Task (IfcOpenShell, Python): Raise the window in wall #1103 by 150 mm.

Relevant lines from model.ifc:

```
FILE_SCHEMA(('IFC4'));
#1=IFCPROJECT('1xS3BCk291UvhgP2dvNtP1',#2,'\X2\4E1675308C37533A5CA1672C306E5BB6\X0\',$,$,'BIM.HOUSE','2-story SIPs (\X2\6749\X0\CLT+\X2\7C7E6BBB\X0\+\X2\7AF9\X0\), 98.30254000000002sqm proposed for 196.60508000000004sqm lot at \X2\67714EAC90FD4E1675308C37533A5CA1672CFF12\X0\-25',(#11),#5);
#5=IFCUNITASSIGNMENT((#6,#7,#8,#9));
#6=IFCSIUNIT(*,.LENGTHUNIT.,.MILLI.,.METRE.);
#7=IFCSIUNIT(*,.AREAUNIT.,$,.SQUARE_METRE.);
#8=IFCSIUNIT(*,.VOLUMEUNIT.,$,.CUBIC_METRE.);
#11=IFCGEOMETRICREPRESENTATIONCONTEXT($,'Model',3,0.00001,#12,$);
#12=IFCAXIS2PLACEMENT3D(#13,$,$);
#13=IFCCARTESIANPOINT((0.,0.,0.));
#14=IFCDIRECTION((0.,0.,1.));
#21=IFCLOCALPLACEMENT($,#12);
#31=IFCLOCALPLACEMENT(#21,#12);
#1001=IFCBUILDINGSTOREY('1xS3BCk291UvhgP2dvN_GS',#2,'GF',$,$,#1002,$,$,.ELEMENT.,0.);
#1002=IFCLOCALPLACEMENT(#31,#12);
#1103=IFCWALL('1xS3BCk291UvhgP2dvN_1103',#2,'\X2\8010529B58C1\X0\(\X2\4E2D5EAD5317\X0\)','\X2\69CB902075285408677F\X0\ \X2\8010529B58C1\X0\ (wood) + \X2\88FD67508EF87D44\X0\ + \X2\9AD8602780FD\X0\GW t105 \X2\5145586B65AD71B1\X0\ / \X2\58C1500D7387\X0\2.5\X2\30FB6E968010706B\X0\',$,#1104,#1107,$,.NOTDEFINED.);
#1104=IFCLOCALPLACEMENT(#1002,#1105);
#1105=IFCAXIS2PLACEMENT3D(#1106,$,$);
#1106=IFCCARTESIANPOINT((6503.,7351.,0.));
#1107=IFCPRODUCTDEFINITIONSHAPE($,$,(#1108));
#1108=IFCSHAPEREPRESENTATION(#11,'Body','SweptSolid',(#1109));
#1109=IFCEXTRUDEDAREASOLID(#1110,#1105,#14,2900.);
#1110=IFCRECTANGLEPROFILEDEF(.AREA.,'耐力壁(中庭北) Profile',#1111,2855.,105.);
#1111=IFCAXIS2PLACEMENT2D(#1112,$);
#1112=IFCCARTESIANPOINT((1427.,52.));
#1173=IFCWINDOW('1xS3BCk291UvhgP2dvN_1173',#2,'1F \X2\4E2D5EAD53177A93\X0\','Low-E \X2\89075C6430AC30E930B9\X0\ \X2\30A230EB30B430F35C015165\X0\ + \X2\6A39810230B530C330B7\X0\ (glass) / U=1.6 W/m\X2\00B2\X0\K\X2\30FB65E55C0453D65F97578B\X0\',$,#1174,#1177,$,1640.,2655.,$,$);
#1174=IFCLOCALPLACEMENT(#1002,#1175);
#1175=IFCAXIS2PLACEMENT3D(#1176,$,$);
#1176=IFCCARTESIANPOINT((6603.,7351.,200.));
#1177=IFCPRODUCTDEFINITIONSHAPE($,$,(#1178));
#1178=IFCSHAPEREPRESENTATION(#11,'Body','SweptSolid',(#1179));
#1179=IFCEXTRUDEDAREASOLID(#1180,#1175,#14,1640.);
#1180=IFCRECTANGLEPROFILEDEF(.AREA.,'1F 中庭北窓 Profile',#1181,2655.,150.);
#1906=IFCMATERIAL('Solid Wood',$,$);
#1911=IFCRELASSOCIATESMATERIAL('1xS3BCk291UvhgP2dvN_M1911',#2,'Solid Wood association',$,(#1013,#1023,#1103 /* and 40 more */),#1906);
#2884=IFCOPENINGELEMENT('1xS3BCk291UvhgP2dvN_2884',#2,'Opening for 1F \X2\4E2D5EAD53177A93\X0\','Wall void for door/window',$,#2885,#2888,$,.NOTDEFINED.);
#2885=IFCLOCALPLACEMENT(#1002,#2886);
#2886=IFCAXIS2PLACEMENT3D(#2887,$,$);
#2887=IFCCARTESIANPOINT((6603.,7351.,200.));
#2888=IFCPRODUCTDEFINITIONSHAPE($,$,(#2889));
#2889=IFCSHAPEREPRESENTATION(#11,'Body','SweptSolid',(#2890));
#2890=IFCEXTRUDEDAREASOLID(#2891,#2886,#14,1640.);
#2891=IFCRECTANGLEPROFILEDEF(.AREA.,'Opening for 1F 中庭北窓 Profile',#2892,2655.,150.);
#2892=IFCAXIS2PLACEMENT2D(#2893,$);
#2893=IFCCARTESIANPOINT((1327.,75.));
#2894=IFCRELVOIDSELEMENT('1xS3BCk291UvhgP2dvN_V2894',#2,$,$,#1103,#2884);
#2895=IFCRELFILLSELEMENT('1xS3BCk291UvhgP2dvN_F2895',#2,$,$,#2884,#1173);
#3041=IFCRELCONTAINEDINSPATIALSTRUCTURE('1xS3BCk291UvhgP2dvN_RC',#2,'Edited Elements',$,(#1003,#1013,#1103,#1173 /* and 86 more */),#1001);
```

```python
import numpy as np
import ifcopenshell
import ifcopenshell.api.geometry
import ifcopenshell.util.placement
import ifcopenshell.util.unit

model = ifcopenshell.open("model.ifc")
unit_scale = ifcopenshell.util.unit.calculate_unit_scale(model)

window = model.by_guid("1xS3BCk291UvhgP2dvN_1173")
opening = window.FillsVoids[0].RelatingOpeningElement
dz = 0.15 / unit_scale

shift = np.array([0.0, 0.0, dz])
# The window is not placed relative to its opening, so move both.
for product in (opening, window):
    matrix = ifcopenshell.util.placement.get_local_placement(product.ObjectPlacement)
    matrix[:3, 3] += shift
    ifcopenshell.api.geometry.edit_object_placement(model, product=product, matrix=matrix, is_si=False)

print(f"moved by {dz * unit_scale:+.3f} m")

model.write("model_edited.ifc")
```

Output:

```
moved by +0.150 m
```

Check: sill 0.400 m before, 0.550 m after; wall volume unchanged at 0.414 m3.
